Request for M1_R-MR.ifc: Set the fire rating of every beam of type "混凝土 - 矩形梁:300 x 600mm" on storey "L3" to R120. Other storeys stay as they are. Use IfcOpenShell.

First a look at what the model holds.

```python
import ifcopenshell
import ifcopenshell.util.element

model = ifcopenshell.open("M1_R-MR.ifc")
print(model.schema)
storey = next(s for s in model.by_type("IfcBuildingStorey") if s.Name == "L3")
beams = [e for e in ifcopenshell.util.element.get_decomposition(storey) if e.is_a("IfcBeam")]
seen = {}
for e in beams:
    element_type = ifcopenshell.util.element.get_type(e)
    key = (element_type.Name if element_type != e and element_type else None, ifcopenshell.util.element.get_pset(e, "Pset_BeamCommon", "FireRating"))
    seen[key] = seen.get(key, 0) + 1
for (name, value), count in sorted(seen.items(), key=str):
    print(count, "x", name, "|", value)
```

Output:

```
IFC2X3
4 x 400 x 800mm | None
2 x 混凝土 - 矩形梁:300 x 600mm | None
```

```python
import ifcopenshell
import ifcopenshell.api.pset
import ifcopenshell.util.element

model = ifcopenshell.open("M1_R-MR.ifc")

storey = next(s for s in model.by_type("IfcBuildingStorey") if s.Name == "L3")
beams = [e for e in ifcopenshell.util.element.get_decomposition(storey) if e.is_a("IfcBeam")]

count = 0
for e in beams:
    element_type = ifcopenshell.util.element.get_type(e)
    if element_type in (None, e) or element_type.Name != "混凝土 - 矩形梁:300 x 600mm":
        continue
    # add_pset returns the element's existing set when there is one.
    pset = ifcopenshell.api.pset.add_pset(model, product=e, name="Pset_BeamCommon")
    ifcopenshell.api.pset.edit_pset(model, pset=pset, properties={"FireRating": "R120"})
    count += 1

print(count, "beams updated")

model.write("M1_R-MR-out.ifc")
```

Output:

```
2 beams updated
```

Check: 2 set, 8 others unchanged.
